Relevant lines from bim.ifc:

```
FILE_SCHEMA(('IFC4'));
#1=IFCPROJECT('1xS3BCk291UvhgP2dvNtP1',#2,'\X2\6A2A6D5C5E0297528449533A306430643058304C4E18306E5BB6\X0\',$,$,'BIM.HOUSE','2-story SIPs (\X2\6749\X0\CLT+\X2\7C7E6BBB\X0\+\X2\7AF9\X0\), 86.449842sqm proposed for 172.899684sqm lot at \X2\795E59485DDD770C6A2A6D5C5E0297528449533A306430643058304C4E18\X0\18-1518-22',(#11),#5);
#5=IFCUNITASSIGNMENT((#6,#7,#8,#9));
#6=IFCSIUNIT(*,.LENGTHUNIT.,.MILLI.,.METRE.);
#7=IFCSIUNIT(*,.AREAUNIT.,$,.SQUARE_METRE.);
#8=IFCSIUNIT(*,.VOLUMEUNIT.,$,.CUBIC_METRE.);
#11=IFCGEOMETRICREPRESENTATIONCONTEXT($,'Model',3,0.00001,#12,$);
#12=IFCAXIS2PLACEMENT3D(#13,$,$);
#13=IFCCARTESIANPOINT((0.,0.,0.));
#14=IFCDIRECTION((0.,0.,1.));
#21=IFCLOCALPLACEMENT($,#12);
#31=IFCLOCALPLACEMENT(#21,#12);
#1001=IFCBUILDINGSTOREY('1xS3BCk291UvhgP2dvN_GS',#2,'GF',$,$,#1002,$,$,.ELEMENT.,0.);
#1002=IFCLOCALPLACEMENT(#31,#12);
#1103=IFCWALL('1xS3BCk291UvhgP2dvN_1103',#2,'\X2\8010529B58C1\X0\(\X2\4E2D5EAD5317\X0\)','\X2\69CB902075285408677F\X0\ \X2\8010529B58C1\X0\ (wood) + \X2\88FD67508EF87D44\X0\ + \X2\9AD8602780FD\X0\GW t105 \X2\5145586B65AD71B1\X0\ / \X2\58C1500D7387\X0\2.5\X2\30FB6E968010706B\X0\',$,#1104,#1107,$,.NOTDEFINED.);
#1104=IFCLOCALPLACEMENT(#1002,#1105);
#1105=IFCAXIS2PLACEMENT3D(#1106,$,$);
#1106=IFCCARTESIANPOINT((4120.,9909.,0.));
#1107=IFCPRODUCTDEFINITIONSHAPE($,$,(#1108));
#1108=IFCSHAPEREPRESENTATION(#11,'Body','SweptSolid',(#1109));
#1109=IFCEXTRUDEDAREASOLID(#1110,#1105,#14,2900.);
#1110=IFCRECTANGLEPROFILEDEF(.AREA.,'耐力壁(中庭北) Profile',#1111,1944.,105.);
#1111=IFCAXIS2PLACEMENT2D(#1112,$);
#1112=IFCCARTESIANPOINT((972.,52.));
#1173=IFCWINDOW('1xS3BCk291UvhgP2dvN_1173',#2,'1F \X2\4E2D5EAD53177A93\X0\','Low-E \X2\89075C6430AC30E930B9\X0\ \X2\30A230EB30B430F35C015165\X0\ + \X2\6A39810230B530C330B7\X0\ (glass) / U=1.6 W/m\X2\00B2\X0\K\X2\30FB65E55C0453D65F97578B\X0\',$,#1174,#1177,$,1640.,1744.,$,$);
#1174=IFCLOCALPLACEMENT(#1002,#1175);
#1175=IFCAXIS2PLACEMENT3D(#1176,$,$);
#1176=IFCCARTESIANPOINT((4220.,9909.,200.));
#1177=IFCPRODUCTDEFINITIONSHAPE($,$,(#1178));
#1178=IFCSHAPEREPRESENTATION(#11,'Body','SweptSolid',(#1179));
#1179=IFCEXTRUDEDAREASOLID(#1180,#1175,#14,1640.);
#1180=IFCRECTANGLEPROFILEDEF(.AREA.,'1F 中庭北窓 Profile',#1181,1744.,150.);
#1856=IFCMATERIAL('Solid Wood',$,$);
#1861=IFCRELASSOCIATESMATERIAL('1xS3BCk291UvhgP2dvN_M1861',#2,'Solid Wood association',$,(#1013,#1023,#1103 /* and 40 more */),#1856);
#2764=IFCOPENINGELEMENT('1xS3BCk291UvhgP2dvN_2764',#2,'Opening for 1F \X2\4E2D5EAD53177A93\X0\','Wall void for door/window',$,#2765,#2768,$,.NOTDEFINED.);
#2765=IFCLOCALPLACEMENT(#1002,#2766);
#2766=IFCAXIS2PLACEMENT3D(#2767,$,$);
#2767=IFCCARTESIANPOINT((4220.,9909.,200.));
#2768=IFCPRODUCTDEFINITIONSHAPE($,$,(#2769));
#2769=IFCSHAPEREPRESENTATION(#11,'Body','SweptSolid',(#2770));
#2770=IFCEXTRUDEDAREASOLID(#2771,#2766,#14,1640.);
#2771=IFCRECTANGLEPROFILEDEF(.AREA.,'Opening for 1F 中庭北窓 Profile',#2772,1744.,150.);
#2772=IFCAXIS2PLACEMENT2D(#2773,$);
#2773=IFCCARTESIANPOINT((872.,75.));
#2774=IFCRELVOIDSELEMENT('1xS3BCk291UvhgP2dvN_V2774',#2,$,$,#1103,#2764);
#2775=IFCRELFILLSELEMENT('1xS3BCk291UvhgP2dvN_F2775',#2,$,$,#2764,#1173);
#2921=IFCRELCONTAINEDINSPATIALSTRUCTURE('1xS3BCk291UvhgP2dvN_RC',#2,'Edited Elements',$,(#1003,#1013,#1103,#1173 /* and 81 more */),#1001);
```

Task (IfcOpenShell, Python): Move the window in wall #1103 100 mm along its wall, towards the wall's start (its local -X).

```python
import ifcopenshell
import ifcopenshell.api.geometry
import ifcopenshell.util.placement
import ifcopenshell.util.unit

model = ifcopenshell.open("bim.ifc")
unit_scale = ifcopenshell.util.unit.calculate_unit_scale(model)

window = model.by_guid("1xS3BCk291UvhgP2dvN_1173")
opening = window.FillsVoids[0].RelatingOpeningElement
wall = opening.VoidsElements[0].RelatingBuildingElement

wall_matrix = ifcopenshell.util.placement.get_local_placement(wall.ObjectPlacement)
shift = wall_matrix[:3, 0] * -0.1 / unit_scale
before = ifcopenshell.util.placement.get_local_placement(window.ObjectPlacement)[:3, 3].copy()

# The window is not placed relative to its opening, so move both.
for product in (opening, window):
    matrix = ifcopenshell.util.placement.get_local_placement(product.ObjectPlacement)
    matrix[:3, 3] += shift
    ifcopenshell.api.geometry.edit_object_placement(model, product=product, matrix=matrix, is_si=False)

after = ifcopenshell.util.placement.get_local_placement(window.ObjectPlacement)[:3, 3]
print("window moved by", (after - before).round(3) + 0.0)

model.write("bim_edited.ifc")
```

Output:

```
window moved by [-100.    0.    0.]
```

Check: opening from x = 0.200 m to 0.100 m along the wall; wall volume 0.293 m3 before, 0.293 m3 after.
